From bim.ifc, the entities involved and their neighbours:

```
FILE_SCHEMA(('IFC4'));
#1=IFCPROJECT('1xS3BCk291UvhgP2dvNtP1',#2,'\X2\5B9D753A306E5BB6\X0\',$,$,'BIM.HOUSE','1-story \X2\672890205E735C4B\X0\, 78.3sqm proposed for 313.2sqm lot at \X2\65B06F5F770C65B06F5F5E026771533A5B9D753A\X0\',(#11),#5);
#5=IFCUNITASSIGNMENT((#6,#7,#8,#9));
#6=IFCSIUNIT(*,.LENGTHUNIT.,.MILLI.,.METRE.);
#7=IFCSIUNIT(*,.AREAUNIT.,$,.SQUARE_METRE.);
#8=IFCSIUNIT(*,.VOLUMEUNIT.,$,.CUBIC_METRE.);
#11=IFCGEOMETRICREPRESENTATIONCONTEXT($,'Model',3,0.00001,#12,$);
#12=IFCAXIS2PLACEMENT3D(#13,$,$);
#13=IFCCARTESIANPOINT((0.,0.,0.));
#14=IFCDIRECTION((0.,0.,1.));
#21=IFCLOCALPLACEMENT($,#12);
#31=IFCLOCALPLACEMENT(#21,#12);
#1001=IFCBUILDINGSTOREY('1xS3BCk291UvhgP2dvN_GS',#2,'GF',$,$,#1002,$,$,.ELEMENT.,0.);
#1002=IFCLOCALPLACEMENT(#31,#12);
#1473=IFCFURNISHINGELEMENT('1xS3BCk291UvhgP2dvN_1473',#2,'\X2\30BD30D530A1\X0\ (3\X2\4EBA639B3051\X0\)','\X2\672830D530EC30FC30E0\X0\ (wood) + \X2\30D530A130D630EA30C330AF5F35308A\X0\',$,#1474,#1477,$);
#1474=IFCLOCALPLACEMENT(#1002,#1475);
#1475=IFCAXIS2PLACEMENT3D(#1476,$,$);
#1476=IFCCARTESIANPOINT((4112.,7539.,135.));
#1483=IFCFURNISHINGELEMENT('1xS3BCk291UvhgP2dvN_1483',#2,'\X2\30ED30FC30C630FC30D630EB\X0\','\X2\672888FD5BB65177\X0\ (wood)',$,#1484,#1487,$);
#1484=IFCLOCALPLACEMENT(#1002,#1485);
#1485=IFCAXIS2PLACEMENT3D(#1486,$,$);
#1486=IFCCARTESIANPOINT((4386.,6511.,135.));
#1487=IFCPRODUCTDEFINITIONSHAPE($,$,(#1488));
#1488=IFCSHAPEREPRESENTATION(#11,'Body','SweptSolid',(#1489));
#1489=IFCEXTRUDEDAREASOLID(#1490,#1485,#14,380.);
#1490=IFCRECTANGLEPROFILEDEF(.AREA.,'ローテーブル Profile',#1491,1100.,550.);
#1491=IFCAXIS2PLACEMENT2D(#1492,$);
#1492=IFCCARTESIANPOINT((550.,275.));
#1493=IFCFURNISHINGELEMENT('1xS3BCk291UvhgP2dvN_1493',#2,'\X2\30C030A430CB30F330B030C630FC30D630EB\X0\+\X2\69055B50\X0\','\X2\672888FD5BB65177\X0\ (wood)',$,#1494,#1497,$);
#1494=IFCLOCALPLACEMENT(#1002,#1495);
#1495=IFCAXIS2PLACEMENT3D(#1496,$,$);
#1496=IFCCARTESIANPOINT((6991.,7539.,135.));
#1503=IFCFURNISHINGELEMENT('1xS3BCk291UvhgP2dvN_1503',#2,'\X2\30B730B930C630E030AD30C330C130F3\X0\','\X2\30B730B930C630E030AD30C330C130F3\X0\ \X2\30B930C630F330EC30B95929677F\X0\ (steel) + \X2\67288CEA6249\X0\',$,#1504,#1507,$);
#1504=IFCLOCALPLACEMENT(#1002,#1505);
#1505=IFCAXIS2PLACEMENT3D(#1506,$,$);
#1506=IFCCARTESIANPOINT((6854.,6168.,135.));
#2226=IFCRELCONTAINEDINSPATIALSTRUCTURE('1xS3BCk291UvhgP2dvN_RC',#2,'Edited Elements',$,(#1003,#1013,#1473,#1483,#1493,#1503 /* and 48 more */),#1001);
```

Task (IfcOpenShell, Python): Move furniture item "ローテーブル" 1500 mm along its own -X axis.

```python
import ifcopenshell
import ifcopenshell.api.geometry
import ifcopenshell.util.placement

model = ifcopenshell.open("bim.ifc")

item = model.by_id(1483)
matrix = ifcopenshell.util.placement.get_local_placement(item.ObjectPlacement)
matrix[:3, 3] -= matrix[:3, 0] * 1500.0
ifcopenshell.api.geometry.edit_object_placement(model, product=item, matrix=matrix, is_si=False)

print(ifcopenshell.util.placement.get_local_placement(item.ObjectPlacement).round(3) + 0.0)

model.write("bim_rev.ifc")
```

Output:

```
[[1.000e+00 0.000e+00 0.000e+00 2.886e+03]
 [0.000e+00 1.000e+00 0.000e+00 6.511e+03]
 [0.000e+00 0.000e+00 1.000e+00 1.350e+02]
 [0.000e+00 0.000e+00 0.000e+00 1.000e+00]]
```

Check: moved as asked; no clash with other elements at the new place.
